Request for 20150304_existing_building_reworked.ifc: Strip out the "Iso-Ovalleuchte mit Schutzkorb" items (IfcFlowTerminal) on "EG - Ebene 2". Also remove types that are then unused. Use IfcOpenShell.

First a look at what the model holds.

```python
import ifcopenshell
import ifcopenshell.util.element

model = ifcopenshell.open("20150304_existing_building_reworked.ifc")
print(model.schema)
storey = next(s for s in model.by_type("IfcBuildingStorey") if s.Name == "EG - Ebene 2")
terminals = [e for e in ifcopenshell.util.element.get_decomposition(storey) if e.is_a("IfcFlowTerminal")]
seen = {}
for e in terminals:
    element_type = ifcopenshell.util.element.get_type(e)
    name = element_type.Name if element_type not in (None, e) else None
    seen[name] = seen.get(name, 0) + 1
for name, count in sorted(seen.items(), key=str):
    print(count, "x", name)
```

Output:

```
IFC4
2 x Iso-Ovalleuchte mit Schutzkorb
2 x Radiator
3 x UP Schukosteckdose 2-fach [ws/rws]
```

```python
import ifcopenshell
import ifcopenshell.api.root
import ifcopenshell.util.element

model = ifcopenshell.open("20150304_existing_building_reworked.ifc")

storey = next(s for s in model.by_type("IfcBuildingStorey") if s.Name == "EG - Ebene 2")
terminals = [e for e in ifcopenshell.util.element.get_decomposition(storey) if e.is_a("IfcFlowTerminal")]
targets = [e for e in terminals if (t := ifcopenshell.util.element.get_type(e)) not in (None, e) and t.Name == "Iso-Ovalleuchte mit Schutzkorb"]
types = {ifcopenshell.util.element.get_type(e) for e in targets} - {None, *targets}

for e in targets:
    ifcopenshell.api.root.remove_product(model, product=e)
print(len(targets), "removed")

unused = [t for t in types if not ifcopenshell.util.element.get_types(t)]
for t in unused:
    ifcopenshell.api.root.remove_product(model, product=t)
print(len(unused), "unused types removed")

model.write("20150304_existing_building_reworked-out.ifc")
```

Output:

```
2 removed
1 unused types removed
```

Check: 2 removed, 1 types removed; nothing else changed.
